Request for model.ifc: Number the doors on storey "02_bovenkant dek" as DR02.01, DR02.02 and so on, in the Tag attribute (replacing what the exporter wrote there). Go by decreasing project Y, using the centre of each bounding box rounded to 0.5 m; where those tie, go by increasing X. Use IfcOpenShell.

First a look at what the model holds.

```python
import ifcopenshell
import ifcopenshell.util.element
import ifcopenshell.util.placement

model = ifcopenshell.open("model.ifc")
print(model.schema)
storey = next(s for s in model.by_type("IfcBuildingStorey") if s.Name == "02_bovenkant dek")
doors = [e for e in ifcopenshell.util.element.get_decomposition(storey) if e.is_a("IfcDoor")]
for e in sorted(doors, key=lambda e: e.id()):
    origin = ifcopenshell.util.placement.get_local_placement(e.ObjectPlacement)[:3, 3]
    print(e.id(), e.Tag, e.Name, origin.round(2) + 0.0, sep=" | ")
```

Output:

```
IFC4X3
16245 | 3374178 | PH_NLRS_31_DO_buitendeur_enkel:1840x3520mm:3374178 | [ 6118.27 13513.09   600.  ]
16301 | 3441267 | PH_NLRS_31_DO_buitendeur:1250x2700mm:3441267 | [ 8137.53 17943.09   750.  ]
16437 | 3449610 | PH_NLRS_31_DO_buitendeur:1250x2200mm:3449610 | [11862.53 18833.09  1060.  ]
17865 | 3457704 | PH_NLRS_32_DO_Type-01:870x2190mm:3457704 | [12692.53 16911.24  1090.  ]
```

```python
import ifcopenshell
import ifcopenshell.geom
import ifcopenshell.util.element
import ifcopenshell.util.shape

model = ifcopenshell.open("model.ifc")
settings = ifcopenshell.geom.settings()
settings.set("use-world-coords", True)


def centre(element):
    shape = ifcopenshell.geom.create_shape(settings, element)
    return ifcopenshell.util.shape.get_bbox_centroid(shape.geometry)


storey = next(s for s in model.by_type("IfcBuildingStorey") if s.Name == "02_bovenkant dek")
doors = [e for e in ifcopenshell.util.element.get_decomposition(storey) if e.is_a("IfcDoor")]

# Insertion points can sit at a corner or the storey origin, so sort by the geometry (in metres).
centres = {e: centre(e) for e in doors}
doors.sort(key=lambda e: (-round(centres[e][1] / 0.5), centres[e][0]))

for i, e in enumerate(doors, start=1):
    number = f"DR02.{i:02d}"
    e.Tag = number
    print(e.id(), number)

model.write("model_v2.ifc")
```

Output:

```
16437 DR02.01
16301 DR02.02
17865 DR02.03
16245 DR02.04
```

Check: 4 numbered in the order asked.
